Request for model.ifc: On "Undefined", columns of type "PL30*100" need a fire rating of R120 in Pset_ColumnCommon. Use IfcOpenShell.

First a look at what the model holds.

```python
import ifcopenshell
import ifcopenshell.util.element

model = ifcopenshell.open("model.ifc")
print(model.schema)
storey = next(s for s in model.by_type("IfcBuildingStorey") if s.Name == "Undefined")
columns = [e for e in ifcopenshell.util.element.get_decomposition(storey) if e.is_a("IfcColumn")]
seen = {}
for e in columns:
    element_type = ifcopenshell.util.element.get_type(e)
    key = (element_type.Name if element_type != e and element_type else None, ifcopenshell.util.element.get_pset(e, "Pset_ColumnCommon", "FireRating"))
    seen[key] = seen.get(key, 0) + 1
for (name, value), count in sorted(seen.items(), key=str):
    print(count, "x", name, "|", value)
```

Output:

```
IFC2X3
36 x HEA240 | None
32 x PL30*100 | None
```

```python
import ifcopenshell
import ifcopenshell.api.pset
import ifcopenshell.util.element

model = ifcopenshell.open("model.ifc")

storey = next(s for s in model.by_type("IfcBuildingStorey") if s.Name == "Undefined")
columns = [e for e in ifcopenshell.util.element.get_decomposition(storey) if e.is_a("IfcColumn")]

count = 0
for e in columns:
    element_type = ifcopenshell.util.element.get_type(e)
    if element_type in (None, e) or element_type.Name != "PL30*100":
        continue
    # add_pset returns the element's existing set when there is one.
    pset = ifcopenshell.api.pset.add_pset(model, product=e, name="Pset_ColumnCommon")
    ifcopenshell.api.pset.edit_pset(model, pset=pset, properties={"FireRating": "R120"})
    count += 1

print(count, "columns updated")

model.write("model_edited.ifc")
```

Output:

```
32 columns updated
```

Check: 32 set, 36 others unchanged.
